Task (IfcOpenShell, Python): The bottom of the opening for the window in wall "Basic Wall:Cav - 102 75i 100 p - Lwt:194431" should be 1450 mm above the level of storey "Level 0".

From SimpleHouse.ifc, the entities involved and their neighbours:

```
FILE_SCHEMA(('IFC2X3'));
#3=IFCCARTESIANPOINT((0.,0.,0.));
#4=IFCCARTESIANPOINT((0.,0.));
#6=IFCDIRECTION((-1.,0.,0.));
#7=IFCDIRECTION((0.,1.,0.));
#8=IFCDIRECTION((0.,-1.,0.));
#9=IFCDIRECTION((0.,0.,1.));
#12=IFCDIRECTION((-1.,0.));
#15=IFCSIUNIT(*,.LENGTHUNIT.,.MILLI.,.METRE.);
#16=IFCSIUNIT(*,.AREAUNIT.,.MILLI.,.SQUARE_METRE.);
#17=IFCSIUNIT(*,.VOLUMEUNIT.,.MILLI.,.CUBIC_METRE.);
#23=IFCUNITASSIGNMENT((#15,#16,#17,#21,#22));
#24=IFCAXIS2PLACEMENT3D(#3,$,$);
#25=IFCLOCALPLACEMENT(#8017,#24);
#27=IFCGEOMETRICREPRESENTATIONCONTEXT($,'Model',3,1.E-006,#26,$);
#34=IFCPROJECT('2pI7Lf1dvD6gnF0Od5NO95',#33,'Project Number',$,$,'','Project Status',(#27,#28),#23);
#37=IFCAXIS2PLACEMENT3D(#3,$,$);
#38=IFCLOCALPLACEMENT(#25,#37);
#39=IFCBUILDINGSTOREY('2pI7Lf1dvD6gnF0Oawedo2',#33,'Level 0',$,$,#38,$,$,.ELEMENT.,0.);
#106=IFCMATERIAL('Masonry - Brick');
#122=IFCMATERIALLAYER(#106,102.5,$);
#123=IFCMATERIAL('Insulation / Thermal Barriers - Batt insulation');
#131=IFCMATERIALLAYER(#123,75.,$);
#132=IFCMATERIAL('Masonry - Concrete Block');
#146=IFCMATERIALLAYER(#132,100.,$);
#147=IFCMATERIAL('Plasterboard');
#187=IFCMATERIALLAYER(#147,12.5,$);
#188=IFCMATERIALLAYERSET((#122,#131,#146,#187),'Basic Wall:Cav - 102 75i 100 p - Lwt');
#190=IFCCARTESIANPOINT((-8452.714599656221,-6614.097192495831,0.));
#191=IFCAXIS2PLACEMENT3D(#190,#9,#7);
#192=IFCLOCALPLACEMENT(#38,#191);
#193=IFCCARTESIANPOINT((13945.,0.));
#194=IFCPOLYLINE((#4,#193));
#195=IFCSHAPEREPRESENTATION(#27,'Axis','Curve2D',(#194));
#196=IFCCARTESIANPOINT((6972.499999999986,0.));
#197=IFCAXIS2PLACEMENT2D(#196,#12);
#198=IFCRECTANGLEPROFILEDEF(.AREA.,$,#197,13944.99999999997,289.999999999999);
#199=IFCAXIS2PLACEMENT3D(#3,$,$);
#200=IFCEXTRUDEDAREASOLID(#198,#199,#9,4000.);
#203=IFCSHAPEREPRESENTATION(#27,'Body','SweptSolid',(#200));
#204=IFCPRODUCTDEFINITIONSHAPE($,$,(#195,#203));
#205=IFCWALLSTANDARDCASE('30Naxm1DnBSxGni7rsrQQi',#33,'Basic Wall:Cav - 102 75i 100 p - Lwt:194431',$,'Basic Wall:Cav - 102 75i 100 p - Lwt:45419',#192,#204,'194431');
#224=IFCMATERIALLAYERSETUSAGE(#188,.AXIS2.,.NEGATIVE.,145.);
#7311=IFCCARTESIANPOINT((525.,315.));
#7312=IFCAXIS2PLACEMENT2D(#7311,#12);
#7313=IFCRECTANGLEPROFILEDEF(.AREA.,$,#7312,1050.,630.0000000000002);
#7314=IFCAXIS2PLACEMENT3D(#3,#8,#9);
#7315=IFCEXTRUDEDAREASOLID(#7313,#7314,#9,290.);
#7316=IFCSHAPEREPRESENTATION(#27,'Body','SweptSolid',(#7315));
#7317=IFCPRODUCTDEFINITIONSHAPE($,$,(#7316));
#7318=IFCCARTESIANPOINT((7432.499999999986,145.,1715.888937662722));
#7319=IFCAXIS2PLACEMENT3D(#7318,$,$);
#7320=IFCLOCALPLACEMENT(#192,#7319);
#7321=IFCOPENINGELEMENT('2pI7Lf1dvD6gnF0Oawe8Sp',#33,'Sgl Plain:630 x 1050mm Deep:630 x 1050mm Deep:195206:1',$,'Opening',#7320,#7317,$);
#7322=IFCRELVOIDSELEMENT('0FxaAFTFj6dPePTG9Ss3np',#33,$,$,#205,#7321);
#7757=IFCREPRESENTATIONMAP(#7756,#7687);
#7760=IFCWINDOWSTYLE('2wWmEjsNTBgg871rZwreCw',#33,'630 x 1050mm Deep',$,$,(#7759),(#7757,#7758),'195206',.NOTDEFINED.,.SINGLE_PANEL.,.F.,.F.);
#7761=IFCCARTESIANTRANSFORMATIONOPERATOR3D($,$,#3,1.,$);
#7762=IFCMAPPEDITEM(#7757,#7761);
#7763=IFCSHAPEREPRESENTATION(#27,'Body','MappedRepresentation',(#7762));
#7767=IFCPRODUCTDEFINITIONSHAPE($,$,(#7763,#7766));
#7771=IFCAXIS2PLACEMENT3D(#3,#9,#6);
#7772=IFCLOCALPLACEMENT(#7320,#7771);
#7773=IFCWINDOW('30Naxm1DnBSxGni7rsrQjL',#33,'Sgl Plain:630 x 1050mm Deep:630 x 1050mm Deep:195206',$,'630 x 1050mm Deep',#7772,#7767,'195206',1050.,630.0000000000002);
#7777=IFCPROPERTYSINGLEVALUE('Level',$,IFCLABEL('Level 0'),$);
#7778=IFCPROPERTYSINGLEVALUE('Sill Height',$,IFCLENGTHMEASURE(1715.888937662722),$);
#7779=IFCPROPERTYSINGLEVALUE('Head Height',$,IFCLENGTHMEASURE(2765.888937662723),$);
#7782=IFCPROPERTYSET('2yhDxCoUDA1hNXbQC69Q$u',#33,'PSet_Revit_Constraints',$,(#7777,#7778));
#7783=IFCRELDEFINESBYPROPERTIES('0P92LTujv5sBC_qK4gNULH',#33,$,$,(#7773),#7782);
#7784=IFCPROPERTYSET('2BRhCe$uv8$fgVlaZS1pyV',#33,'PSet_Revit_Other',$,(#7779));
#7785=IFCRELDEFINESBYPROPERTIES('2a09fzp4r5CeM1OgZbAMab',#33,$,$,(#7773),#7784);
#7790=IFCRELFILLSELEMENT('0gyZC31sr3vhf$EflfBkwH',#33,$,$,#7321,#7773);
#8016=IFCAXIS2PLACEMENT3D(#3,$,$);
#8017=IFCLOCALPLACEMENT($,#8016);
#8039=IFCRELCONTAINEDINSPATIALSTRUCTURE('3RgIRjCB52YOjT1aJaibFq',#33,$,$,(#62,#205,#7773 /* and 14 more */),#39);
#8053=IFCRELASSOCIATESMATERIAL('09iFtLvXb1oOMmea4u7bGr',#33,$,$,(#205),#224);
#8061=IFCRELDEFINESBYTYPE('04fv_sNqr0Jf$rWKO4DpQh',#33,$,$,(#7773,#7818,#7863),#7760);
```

```python
import numpy as np
import ifcopenshell
import ifcopenshell.api.geometry
import ifcopenshell.api.pset
import ifcopenshell.geom
import ifcopenshell.util.element
import ifcopenshell.util.placement
import ifcopenshell.util.shape
import ifcopenshell.util.unit

model = ifcopenshell.open("SimpleHouse.ifc")
unit_scale = ifcopenshell.util.unit.calculate_unit_scale(model)

window = model.by_guid("30Naxm1DnBSxGni7rsrQjL")
opening = window.FillsVoids[0].RelatingOpeningElement
storey = ifcopenshell.util.element.get_container(window, ifc_class="IfcBuildingStorey")
level = ifcopenshell.util.placement.get_local_placement(storey.ObjectPlacement)[2, 3]

# The opening's origin need not be at the sill, so measure its lowest point.
shape = ifcopenshell.geom.create_shape(ifcopenshell.geom.settings(), opening)
bottom = ifcopenshell.util.shape.get_shape_bottom_elevation(shape, shape.geometry) / unit_scale
dz = level + 1.45 / unit_scale - bottom

shift = np.array([0.0, 0.0, dz])
# The window is placed relative to its opening, so it follows when the opening moves.
matrix = ifcopenshell.util.placement.get_local_placement(opening.ObjectPlacement)
matrix[:3, 3] += shift
ifcopenshell.api.geometry.edit_object_placement(
    model, product=opening, matrix=matrix, is_si=False, should_transform_children=True
)

# Keep the stored heights in step.
pset = model.by_id(ifcopenshell.util.element.get_pset(window, "PSet_Revit_Constraints", should_inherit=False)["id"])
ifcopenshell.api.pset.edit_pset(model, pset=pset, properties={
    "Sill Height": model.create_entity("IfcLengthMeasure", ifcopenshell.util.element.get_pset(window, "PSet_Revit_Constraints", "Sill Height") + dz),
})
pset = model.by_id(ifcopenshell.util.element.get_pset(window, "PSet_Revit_Other", should_inherit=False)["id"])
ifcopenshell.api.pset.edit_pset(model, pset=pset, properties={
    "Head Height": model.create_entity("IfcLengthMeasure", ifcopenshell.util.element.get_pset(window, "PSet_Revit_Other", "Head Height") + dz),
})

print(f"moved by {dz * unit_scale:+.3f} m")

model.write("SimpleHouse_v2.ifc")
```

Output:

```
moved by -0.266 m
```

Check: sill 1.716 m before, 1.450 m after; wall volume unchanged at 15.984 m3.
